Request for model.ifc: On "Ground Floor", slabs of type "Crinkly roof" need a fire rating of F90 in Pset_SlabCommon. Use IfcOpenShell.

First a look at what the model holds.

```python
import ifcopenshell
import ifcopenshell.util.element

model = ifcopenshell.open("model.ifc")
print(model.schema)
storey = next(s for s in model.by_type("IfcBuildingStorey") if s.Name == "Ground Floor")
slabs = [e for e in ifcopenshell.util.element.get_decomposition(storey) if e.is_a("IfcSlab")]
seen = {}
for e in slabs:
    element_type = ifcopenshell.util.element.get_type(e)
    key = (element_type.Name if element_type != e and element_type else None, ifcopenshell.util.element.get_pset(e, "Pset_SlabCommon", "FireRating"))
    seen[key] = seen.get(key, 0) + 1
for (name, value), count in sorted(seen.items(), key=str):
    print(count, "x", name, "|", value)
```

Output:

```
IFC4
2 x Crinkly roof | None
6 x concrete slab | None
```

```python
import ifcopenshell
import ifcopenshell.api.pset
import ifcopenshell.util.element

model = ifcopenshell.open("model.ifc")

storey = next(s for s in model.by_type("IfcBuildingStorey") if s.Name == "Ground Floor")
slabs = [e for e in ifcopenshell.util.element.get_decomposition(storey) if e.is_a("IfcSlab")]

count = 0
for e in slabs:
    element_type = ifcopenshell.util.element.get_type(e)
    if element_type in (None, e) or element_type.Name != "Crinkly roof":
        continue
    # add_pset returns the element's existing set when there is one.
    pset = ifcopenshell.api.pset.add_pset(model, product=e, name="Pset_SlabCommon")
    ifcopenshell.api.pset.edit_pset(model, pset=pset, properties={"FireRating": "F90"})
    count += 1

print(count, "slabs updated")

model.write("model_v2.ifc")
```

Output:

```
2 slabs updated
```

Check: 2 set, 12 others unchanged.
